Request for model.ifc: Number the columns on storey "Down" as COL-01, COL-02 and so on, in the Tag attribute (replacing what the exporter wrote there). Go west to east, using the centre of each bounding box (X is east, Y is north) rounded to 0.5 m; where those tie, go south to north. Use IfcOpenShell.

First a look at what the model holds.

```python
import ifcopenshell
import ifcopenshell.util.element
import ifcopenshell.util.placement

model = ifcopenshell.open("model.ifc")
print(model.schema)
storey = next(s for s in model.by_type("IfcBuildingStorey") if s.Name == "Down")
columns = [e for e in ifcopenshell.util.element.get_decomposition(storey) if e.is_a("IfcColumn")]
for e in sorted(columns, key=lambda e: e.id()):
    origin = ifcopenshell.util.placement.get_local_placement(e.ObjectPlacement)[:3, 3]
    print(e.id(), e.Tag, e.Name, origin.round(2) + 0.0, sep=" | ")
```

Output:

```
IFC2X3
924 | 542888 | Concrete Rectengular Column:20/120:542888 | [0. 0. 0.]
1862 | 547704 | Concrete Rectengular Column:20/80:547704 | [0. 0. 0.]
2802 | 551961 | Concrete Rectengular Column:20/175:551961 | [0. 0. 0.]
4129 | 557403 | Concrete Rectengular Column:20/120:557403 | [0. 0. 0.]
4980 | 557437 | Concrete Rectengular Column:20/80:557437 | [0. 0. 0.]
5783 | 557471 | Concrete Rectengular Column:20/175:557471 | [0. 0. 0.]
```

```python
import ifcopenshell
import ifcopenshell.geom
import ifcopenshell.util.element
import ifcopenshell.util.shape

model = ifcopenshell.open("model.ifc")
settings = ifcopenshell.geom.settings()
settings.set("use-world-coords", True)


def centre(element):
    shape = ifcopenshell.geom.create_shape(settings, element)
    return ifcopenshell.util.shape.get_bbox_centroid(shape.geometry)


storey = next(s for s in model.by_type("IfcBuildingStorey") if s.Name == "Down")
columns = [e for e in ifcopenshell.util.element.get_decomposition(storey) if e.is_a("IfcColumn")]

# Insertion points can sit at a corner or the storey origin, so sort by the geometry (in metres).
centres = {e: centre(e) for e in columns}
columns.sort(key=lambda e: (round(centres[e][0] / 0.5), centres[e][1]))

for i, e in enumerate(columns, start=1):
    number = f"COL-{i:02d}"
    e.Tag = number
    print(e.id(), number)

model.write("model_rev.ifc")
```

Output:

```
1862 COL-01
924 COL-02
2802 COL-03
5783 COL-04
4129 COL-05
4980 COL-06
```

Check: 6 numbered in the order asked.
